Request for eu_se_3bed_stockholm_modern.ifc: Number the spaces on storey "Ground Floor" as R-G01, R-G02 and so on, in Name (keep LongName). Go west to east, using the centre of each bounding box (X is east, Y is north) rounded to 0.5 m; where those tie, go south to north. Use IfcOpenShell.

First a look at what the model holds.

```python
import ifcopenshell
import ifcopenshell.util.element
import ifcopenshell.util.placement

model = ifcopenshell.open("eu_se_3bed_stockholm_modern.ifc")
print(model.schema)
storey = next(s for s in model.by_type("IfcBuildingStorey") if s.Name == "Ground Floor")
spaces = [e for e in ifcopenshell.util.element.get_decomposition(storey) if e.is_a("IfcSpace")]
for e in sorted(spaces, key=lambda e: e.id()):
    origin = ifcopenshell.util.placement.get_local_placement(e.ObjectPlacement)[:3, 3]
    print(e.id(), e.Name, e.LongName, origin.round(2) + 0.0, sep=" | ")
```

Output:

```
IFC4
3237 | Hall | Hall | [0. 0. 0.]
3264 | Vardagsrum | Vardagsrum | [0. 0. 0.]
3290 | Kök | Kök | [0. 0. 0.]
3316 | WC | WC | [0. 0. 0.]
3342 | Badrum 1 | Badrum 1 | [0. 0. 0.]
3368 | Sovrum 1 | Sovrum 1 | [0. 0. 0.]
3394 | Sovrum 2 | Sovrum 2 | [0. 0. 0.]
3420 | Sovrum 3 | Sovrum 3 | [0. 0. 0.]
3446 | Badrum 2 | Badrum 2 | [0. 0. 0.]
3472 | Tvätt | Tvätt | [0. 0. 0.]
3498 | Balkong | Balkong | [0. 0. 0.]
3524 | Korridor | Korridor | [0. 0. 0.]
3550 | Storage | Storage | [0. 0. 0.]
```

```python
import ifcopenshell
import ifcopenshell.geom
import ifcopenshell.util.element
import ifcopenshell.util.shape

model = ifcopenshell.open("eu_se_3bed_stockholm_modern.ifc")
settings = ifcopenshell.geom.settings()
settings.set("use-world-coords", True)


def centre(element):
    shape = ifcopenshell.geom.create_shape(settings, element)
    return ifcopenshell.util.shape.get_bbox_centroid(shape.geometry)


storey = next(s for s in model.by_type("IfcBuildingStorey") if s.Name == "Ground Floor")
spaces = [e for e in ifcopenshell.util.element.get_decomposition(storey) if e.is_a("IfcSpace")]

# Insertion points can sit at a corner or the storey origin, so sort by the geometry (in metres).
centres = {e: centre(e) for e in spaces}
spaces.sort(key=lambda e: (round(centres[e][0] / 0.5), centres[e][1]))

for i, e in enumerate(spaces, start=1):
    number = f"R-G{i:02d}"
    e.Name = number
    print(e.id(), number)

model.write("eu_se_3bed_stockholm_modern_edited.ifc")
```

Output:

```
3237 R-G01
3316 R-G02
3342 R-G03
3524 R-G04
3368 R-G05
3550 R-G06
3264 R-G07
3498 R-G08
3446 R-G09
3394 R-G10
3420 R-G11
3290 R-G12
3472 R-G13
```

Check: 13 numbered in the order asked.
